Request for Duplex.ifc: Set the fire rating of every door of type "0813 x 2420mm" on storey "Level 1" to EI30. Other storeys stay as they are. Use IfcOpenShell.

First a look at what the model holds.

```python
import ifcopenshell
import ifcopenshell.util.element

model = ifcopenshell.open("Duplex.ifc")
print(model.schema)
storey = next(s for s in model.by_type("IfcBuildingStorey") if s.Name == "Level 1")
doors = [e for e in ifcopenshell.util.element.get_decomposition(storey) if e.is_a("IfcDoor")]
seen = {}
for e in doors:
    element_type = ifcopenshell.util.element.get_type(e)
    key = (element_type.Name if element_type != e and element_type else None, ifcopenshell.util.element.get_pset(e, "Pset_DoorCommon", "FireRating"))
    seen[key] = seen.get(key, 0) + 1
for (name, value), count in sorted(seen.items(), key=str):
    print(count, "x", name, "|", value)
```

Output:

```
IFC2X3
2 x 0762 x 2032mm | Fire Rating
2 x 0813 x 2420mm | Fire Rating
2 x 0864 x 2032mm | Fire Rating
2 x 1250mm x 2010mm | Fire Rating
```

```python
import ifcopenshell
import ifcopenshell.api.pset
import ifcopenshell.util.element

model = ifcopenshell.open("Duplex.ifc")

storey = next(s for s in model.by_type("IfcBuildingStorey") if s.Name == "Level 1")
doors = [e for e in ifcopenshell.util.element.get_decomposition(storey) if e.is_a("IfcDoor")]

count = 0
for e in doors:
    element_type = ifcopenshell.util.element.get_type(e)
    if element_type in (None, e) or element_type.Name != "0813 x 2420mm":
        continue
    # add_pset returns the element's existing set when there is one.
    pset = ifcopenshell.api.pset.add_pset(model, product=e, name="Pset_DoorCommon")
    ifcopenshell.api.pset.edit_pset(model, pset=pset, properties={"FireRating": "EI30"})
    count += 1

print(count, "doors updated")

model.write("Duplex_v2.ifc")
```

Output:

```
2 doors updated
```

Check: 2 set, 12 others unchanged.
